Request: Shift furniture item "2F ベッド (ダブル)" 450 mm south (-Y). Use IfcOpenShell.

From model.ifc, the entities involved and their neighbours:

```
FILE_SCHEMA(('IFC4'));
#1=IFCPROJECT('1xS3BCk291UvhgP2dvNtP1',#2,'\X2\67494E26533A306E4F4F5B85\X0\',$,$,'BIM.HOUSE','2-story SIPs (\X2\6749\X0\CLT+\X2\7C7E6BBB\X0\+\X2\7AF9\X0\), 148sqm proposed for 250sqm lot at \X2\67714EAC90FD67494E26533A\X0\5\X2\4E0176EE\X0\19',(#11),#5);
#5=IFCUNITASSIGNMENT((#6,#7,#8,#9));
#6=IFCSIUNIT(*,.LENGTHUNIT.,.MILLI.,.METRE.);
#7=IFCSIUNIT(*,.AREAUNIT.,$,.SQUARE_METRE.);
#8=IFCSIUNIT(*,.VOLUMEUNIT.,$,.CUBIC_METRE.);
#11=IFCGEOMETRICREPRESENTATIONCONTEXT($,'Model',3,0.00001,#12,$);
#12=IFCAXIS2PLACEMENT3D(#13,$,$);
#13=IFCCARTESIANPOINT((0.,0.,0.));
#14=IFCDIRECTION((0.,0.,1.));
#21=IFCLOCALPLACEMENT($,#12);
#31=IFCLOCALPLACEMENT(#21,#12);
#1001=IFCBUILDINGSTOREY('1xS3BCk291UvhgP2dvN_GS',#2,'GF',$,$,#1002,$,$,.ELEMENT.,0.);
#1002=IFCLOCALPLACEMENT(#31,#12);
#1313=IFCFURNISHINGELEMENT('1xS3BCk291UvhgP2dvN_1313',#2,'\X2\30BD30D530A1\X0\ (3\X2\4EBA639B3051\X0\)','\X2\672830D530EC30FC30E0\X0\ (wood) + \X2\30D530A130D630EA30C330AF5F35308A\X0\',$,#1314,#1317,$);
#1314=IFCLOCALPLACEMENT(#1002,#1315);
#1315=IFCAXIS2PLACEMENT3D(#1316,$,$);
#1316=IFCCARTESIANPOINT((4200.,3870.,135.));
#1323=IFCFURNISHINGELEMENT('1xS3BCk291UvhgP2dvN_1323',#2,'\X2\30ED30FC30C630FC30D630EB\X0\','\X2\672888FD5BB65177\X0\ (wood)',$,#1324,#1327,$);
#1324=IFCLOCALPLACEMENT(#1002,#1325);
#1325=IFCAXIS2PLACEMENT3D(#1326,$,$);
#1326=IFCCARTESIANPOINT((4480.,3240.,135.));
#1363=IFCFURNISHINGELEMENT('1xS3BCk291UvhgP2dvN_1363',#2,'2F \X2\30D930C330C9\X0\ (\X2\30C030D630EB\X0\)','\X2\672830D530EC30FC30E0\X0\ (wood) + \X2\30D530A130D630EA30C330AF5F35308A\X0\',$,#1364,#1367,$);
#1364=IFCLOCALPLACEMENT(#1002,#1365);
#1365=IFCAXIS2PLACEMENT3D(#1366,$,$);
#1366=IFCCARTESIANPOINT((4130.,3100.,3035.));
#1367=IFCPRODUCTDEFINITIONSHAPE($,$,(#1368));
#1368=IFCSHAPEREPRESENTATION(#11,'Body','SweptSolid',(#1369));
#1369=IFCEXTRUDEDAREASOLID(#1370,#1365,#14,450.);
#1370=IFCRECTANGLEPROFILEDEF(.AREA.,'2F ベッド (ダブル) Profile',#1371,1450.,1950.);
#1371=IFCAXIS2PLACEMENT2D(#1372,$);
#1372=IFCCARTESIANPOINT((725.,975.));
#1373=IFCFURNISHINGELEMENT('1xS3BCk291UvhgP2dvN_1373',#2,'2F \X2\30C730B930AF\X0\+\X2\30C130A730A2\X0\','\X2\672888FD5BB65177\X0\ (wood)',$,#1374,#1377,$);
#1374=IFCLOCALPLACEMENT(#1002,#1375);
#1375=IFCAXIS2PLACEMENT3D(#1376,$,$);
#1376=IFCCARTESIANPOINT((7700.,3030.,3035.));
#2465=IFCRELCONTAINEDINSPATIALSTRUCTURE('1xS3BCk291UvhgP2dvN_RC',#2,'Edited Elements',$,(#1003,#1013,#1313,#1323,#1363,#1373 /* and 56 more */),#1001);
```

```python
import ifcopenshell
import ifcopenshell.api.geometry
import ifcopenshell.util.placement

model = ifcopenshell.open("model.ifc")

item = model.by_guid("1xS3BCk291UvhgP2dvN_1363")
matrix = ifcopenshell.util.placement.get_local_placement(item.ObjectPlacement)
matrix[1, 3] -= 450.0
ifcopenshell.api.geometry.edit_object_placement(model, product=item, matrix=matrix, is_si=False)

print(ifcopenshell.util.placement.get_local_placement(item.ObjectPlacement).round(3) + 0.0)

model.write("model_updated.ifc")
```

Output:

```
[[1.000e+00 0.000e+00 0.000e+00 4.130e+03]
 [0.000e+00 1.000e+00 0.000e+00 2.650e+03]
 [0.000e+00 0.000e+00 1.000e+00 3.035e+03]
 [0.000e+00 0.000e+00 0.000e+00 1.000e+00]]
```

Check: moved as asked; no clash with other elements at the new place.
